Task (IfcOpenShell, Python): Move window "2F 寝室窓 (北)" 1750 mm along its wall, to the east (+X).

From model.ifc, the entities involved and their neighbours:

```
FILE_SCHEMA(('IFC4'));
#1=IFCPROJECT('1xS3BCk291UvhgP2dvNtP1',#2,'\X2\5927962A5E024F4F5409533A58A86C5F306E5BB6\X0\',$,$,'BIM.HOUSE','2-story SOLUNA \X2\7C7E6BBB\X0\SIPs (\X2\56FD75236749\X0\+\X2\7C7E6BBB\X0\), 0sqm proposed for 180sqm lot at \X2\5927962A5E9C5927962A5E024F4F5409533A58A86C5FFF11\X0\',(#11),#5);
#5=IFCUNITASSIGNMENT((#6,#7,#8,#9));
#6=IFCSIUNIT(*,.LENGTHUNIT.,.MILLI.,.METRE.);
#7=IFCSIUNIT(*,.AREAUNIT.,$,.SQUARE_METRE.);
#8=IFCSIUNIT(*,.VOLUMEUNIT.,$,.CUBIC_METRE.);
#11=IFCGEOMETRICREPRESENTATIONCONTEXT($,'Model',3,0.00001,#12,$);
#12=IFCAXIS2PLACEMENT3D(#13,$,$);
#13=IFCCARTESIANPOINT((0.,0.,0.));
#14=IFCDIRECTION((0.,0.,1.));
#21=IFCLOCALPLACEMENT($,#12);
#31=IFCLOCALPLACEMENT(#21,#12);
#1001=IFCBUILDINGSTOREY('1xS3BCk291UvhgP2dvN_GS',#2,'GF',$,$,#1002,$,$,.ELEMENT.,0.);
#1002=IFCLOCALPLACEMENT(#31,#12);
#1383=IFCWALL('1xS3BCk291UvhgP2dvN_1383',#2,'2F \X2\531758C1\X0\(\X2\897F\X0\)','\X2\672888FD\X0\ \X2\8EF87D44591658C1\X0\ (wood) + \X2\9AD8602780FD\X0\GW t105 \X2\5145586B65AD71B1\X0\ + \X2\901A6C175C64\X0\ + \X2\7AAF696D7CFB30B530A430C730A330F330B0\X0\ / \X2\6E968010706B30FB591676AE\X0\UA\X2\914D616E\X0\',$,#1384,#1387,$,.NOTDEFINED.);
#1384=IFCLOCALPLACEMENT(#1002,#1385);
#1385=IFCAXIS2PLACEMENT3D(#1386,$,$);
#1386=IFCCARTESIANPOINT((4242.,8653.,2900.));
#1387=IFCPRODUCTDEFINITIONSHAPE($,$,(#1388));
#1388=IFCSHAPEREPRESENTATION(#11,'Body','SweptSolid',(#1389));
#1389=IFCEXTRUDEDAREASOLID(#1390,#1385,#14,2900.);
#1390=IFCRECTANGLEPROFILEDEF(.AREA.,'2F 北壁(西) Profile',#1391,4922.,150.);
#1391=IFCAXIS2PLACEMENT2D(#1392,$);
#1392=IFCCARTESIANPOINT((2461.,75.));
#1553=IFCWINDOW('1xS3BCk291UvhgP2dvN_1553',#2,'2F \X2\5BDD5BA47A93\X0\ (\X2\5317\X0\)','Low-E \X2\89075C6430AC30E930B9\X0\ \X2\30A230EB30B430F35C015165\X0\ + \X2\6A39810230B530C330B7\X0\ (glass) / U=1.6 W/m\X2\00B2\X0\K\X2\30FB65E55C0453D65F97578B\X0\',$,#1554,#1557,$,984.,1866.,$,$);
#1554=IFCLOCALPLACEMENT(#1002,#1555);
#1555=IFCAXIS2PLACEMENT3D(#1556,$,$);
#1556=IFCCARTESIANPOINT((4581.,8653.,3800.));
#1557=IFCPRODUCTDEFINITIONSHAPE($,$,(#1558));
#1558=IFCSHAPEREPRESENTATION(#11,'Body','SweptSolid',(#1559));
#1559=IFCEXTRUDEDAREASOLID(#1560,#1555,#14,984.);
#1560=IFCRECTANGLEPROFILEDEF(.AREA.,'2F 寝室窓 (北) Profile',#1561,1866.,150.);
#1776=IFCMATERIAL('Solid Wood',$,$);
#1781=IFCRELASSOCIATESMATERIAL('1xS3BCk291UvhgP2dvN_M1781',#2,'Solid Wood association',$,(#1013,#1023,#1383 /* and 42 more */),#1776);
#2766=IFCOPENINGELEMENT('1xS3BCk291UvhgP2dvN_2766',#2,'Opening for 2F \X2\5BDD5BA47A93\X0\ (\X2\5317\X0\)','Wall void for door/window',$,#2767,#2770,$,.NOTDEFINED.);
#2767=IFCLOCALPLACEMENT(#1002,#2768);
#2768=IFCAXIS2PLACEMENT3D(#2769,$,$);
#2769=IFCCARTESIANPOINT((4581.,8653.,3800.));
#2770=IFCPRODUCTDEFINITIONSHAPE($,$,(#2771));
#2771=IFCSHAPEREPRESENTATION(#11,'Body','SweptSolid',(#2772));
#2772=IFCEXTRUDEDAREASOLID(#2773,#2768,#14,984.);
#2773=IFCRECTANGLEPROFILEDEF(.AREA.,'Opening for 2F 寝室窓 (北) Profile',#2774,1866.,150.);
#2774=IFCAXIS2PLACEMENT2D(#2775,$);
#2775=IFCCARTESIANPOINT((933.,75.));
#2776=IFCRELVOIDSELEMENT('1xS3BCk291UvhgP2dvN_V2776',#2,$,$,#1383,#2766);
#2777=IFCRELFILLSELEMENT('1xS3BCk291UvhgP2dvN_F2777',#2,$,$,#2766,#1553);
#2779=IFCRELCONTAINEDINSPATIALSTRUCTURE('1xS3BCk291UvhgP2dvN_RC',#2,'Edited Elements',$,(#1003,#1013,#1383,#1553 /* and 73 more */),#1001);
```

```python
import ifcopenshell
import ifcopenshell.api.geometry
import ifcopenshell.util.placement
import ifcopenshell.util.unit

model = ifcopenshell.open("model.ifc")
unit_scale = ifcopenshell.util.unit.calculate_unit_scale(model)

window = model.by_id(1553)
opening = window.FillsVoids[0].RelatingOpeningElement
wall = opening.VoidsElements[0].RelatingBuildingElement

wall_matrix = ifcopenshell.util.placement.get_local_placement(wall.ObjectPlacement)
shift = wall_matrix[:3, 0] * 1.75 / unit_scale
before = ifcopenshell.util.placement.get_local_placement(window.ObjectPlacement)[:3, 3].copy()

# The window is not placed relative to its opening, so move both.
for product in (opening, window):
    matrix = ifcopenshell.util.placement.get_local_placement(product.ObjectPlacement)
    matrix[:3, 3] += shift
    ifcopenshell.api.geometry.edit_object_placement(model, product=product, matrix=matrix, is_si=False)

after = ifcopenshell.util.placement.get_local_placement(window.ObjectPlacement)[:3, 3]
print("window moved by", (after - before).round(3) + 0.0)

model.write("model_updated.ifc")
```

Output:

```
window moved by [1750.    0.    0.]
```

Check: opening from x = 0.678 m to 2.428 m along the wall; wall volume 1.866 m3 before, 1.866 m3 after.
